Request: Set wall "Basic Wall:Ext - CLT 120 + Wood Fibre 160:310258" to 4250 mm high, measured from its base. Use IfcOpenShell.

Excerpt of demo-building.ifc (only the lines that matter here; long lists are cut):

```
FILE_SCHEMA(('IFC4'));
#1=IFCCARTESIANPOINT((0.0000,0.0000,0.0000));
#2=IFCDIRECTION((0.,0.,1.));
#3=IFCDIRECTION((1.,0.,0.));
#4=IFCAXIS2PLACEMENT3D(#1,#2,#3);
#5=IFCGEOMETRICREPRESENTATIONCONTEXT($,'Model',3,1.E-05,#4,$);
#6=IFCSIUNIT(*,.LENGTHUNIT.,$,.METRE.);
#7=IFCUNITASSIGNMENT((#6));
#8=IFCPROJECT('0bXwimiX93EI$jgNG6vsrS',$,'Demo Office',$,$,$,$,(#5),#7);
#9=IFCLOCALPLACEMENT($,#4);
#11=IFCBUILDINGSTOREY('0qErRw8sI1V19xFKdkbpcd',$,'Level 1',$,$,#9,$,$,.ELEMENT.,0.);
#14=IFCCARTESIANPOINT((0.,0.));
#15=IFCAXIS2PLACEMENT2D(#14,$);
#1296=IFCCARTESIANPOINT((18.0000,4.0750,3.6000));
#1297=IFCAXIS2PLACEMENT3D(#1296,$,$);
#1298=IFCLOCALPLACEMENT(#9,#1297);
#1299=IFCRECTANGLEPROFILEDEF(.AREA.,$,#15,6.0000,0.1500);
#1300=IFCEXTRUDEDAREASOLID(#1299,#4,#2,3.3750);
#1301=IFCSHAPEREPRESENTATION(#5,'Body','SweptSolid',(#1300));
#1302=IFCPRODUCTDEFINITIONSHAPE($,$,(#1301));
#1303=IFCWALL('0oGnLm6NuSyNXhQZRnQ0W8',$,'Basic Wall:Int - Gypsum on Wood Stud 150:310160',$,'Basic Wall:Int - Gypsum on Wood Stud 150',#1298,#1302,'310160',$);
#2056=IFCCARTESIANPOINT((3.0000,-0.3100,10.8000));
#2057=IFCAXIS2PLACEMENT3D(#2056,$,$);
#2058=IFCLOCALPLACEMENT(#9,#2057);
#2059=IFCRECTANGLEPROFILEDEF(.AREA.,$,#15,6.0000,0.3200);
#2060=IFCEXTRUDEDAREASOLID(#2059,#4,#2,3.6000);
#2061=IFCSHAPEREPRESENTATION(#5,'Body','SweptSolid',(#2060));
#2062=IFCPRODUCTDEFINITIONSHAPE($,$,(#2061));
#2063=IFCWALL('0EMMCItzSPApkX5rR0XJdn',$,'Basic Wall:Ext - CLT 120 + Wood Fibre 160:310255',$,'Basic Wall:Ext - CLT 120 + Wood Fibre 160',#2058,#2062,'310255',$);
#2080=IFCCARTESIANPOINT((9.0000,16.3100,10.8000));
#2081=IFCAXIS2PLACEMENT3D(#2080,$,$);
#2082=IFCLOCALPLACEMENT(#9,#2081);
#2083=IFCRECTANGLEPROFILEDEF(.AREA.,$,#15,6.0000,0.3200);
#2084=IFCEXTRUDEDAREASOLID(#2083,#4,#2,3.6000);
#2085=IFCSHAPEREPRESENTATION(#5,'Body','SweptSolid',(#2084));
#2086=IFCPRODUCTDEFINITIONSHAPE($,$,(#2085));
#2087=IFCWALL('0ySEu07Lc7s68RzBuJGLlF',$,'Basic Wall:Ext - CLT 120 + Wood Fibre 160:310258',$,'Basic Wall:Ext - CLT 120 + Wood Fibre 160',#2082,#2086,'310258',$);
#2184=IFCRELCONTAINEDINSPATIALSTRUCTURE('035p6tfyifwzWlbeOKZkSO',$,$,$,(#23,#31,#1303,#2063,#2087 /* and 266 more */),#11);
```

```python
import ifcopenshell
import ifcopenshell.geom
import ifcopenshell.util.shape

model = ifcopenshell.open("demo-building.ifc")
settings = ifcopenshell.geom.settings()


def volume(element):
    """Net volume in cubic metres, openings subtracted."""
    shape = ifcopenshell.geom.create_shape(settings, element)
    return ifcopenshell.util.shape.get_volume(shape.geometry)


wall = model.by_guid("0ySEu07Lc7s68RzBuJGLlF")
before = volume(wall)

body = next(r for r in wall.Representation.Representations if r.RepresentationIdentifier == "Body")
solid = body.Items[0]
old_height = solid.Depth
solid.Depth = 4.25
after = volume(wall)

print(f"height {old_height:g} -> {solid.Depth:g}, volume {before:.3f} -> {after:.3f} m3")

model.write("demo-building-out.ifc")
```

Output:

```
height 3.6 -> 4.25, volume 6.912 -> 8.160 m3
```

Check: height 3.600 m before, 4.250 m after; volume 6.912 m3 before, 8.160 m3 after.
